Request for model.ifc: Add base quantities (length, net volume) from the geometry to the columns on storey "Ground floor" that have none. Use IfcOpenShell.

First a look at what the model holds.

```python
import ifcopenshell
import ifcopenshell.util.element
import ifcopenshell.util.unit

model = ifcopenshell.open("model.ifc")
print(model.schema)
for unit_type in ("LENGTHUNIT", "AREAUNIT", "VOLUMEUNIT"):
    print(unit_type, ifcopenshell.util.unit.calculate_unit_scale(model, unit_type))
storey = next(s for s in model.by_type("IfcBuildingStorey") if s.Name == "Ground floor")
columns = [e for e in ifcopenshell.util.element.get_decomposition(storey) if e.is_a("IfcColumn")]
for e in sorted(columns, key=lambda e: e.id()):
    print(e.id(), e.is_a(), e.Name, list(ifcopenshell.util.element.get_psets(e, qtos_only=True)), sep=" | ")
```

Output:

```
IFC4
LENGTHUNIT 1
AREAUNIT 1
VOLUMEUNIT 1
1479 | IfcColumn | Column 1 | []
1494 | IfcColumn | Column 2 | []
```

```python
import ifcopenshell
import ifcopenshell.api.pset
import ifcopenshell.geom
import ifcopenshell.util.element
import ifcopenshell.util.shape
import ifcopenshell.util.unit

model = ifcopenshell.open("model.ifc")
unit_scale = ifcopenshell.util.unit.calculate_unit_scale(model)
volume_scale = ifcopenshell.util.unit.calculate_unit_scale(model, "VOLUMEUNIT")
settings = ifcopenshell.geom.settings()

storey = next(s for s in model.by_type("IfcBuildingStorey") if s.Name == "Ground floor")
columns = [e for e in ifcopenshell.util.element.get_decomposition(storey) if e.is_a("IfcColumn")]

for e in sorted(columns, key=lambda e: e.id()):
    if ifcopenshell.util.element.get_psets(e, qtos_only=True, should_inherit=False):
        continue
    # Geometry comes back in metres, in the element's own axes.
    shape = ifcopenshell.geom.create_shape(settings, e)
    values = {
        "Length": ifcopenshell.util.shape.get_z(shape.geometry) / unit_scale,
        "NetVolume": ifcopenshell.util.shape.get_volume(shape.geometry) / volume_scale,
    }
    qto = ifcopenshell.api.pset.add_qto(model, product=e, name="Qto_ColumnBaseQuantities")
    ifcopenshell.api.pset.edit_qto(model, qto=qto, properties=values)
    print(e.id(), {k: round(v, 3) for k, v in values.items()})

model.write("model_updated.ifc")
```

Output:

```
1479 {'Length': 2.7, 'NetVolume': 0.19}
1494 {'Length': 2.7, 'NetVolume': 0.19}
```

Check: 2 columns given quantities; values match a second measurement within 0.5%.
